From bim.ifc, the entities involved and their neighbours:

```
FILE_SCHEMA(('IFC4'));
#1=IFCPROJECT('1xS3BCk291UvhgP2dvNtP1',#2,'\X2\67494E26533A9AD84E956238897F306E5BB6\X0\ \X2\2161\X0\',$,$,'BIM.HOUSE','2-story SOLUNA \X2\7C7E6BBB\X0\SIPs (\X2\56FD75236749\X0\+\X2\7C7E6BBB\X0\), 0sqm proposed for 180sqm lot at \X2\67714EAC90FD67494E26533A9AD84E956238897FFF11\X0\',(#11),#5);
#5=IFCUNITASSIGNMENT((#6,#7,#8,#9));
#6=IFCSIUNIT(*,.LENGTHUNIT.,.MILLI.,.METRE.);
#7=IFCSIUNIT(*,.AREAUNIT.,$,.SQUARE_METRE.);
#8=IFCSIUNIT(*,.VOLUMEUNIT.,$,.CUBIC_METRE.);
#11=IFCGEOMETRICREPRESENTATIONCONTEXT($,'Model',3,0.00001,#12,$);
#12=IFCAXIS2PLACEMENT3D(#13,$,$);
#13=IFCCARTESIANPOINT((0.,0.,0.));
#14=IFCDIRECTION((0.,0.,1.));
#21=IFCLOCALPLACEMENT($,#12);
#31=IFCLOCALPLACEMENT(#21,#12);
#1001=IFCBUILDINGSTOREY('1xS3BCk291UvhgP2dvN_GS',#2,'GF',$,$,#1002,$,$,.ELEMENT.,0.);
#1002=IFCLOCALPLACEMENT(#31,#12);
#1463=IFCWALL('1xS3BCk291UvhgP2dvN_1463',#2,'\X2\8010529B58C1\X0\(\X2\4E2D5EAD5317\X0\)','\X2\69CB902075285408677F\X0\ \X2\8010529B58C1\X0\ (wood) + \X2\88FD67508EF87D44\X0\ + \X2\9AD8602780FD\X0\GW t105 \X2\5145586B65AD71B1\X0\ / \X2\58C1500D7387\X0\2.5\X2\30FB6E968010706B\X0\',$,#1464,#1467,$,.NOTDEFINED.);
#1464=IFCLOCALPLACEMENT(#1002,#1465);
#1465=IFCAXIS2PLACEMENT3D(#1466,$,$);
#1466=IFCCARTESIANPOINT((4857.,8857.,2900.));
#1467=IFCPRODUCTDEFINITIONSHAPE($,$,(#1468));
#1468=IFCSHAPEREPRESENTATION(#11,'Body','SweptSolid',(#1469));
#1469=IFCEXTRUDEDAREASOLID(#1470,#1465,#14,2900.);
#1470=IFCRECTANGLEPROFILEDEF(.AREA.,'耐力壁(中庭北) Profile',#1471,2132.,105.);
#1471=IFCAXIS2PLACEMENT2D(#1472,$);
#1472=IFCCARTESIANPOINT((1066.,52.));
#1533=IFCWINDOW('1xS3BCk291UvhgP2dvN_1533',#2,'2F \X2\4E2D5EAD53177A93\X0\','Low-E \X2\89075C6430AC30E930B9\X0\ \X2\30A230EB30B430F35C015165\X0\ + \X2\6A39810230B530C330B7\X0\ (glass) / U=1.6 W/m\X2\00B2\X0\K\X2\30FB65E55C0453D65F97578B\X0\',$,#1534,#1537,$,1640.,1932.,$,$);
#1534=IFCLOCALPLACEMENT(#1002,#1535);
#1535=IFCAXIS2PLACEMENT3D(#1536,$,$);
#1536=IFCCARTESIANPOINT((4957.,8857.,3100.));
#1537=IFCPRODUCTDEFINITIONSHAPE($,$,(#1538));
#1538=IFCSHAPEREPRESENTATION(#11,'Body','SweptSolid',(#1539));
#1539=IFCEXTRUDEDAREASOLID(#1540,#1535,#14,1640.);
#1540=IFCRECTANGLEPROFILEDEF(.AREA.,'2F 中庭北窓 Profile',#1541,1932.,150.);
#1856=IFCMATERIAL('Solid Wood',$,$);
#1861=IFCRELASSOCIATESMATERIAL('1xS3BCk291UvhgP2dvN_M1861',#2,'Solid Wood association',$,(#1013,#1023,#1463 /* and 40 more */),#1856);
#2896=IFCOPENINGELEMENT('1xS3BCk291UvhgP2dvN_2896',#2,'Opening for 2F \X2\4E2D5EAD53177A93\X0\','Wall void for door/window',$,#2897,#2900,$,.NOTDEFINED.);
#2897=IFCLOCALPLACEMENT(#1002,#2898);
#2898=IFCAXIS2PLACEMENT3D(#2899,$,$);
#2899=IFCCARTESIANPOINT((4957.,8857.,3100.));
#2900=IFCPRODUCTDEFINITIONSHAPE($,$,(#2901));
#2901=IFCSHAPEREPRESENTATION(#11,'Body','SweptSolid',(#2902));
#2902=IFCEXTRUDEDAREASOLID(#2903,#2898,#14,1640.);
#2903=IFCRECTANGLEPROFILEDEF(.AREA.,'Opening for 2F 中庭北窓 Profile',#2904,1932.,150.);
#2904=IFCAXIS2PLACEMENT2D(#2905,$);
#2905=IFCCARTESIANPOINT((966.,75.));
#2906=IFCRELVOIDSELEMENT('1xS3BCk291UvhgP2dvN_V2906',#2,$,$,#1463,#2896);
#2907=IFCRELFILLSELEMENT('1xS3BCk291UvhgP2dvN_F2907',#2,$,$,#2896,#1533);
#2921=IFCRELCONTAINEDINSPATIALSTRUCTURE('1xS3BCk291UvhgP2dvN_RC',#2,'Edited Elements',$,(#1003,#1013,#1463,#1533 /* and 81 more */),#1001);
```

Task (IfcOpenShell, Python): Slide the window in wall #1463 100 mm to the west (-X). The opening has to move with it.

```python
import ifcopenshell
import ifcopenshell.api.geometry
import ifcopenshell.util.placement
import ifcopenshell.util.unit

model = ifcopenshell.open("bim.ifc")
unit_scale = ifcopenshell.util.unit.calculate_unit_scale(model)

window = model.by_id(1533)
opening = window.FillsVoids[0].RelatingOpeningElement
wall = opening.VoidsElements[0].RelatingBuildingElement

wall_matrix = ifcopenshell.util.placement.get_local_placement(wall.ObjectPlacement)
shift = wall_matrix[:3, 0] * -0.1 / unit_scale
before = ifcopenshell.util.placement.get_local_placement(window.ObjectPlacement)[:3, 3].copy()

# The window is not placed relative to its opening, so move both.
for product in (opening, window):
    matrix = ifcopenshell.util.placement.get_local_placement(product.ObjectPlacement)
    matrix[:3, 3] += shift
    ifcopenshell.api.geometry.edit_object_placement(model, product=product, matrix=matrix, is_si=False)

after = ifcopenshell.util.placement.get_local_placement(window.ObjectPlacement)[:3, 3]
print("window moved by", (after - before).round(3) + 0.0)

model.write("bim_edited.ifc")
```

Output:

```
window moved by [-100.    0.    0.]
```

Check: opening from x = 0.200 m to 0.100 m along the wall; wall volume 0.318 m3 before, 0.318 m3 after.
